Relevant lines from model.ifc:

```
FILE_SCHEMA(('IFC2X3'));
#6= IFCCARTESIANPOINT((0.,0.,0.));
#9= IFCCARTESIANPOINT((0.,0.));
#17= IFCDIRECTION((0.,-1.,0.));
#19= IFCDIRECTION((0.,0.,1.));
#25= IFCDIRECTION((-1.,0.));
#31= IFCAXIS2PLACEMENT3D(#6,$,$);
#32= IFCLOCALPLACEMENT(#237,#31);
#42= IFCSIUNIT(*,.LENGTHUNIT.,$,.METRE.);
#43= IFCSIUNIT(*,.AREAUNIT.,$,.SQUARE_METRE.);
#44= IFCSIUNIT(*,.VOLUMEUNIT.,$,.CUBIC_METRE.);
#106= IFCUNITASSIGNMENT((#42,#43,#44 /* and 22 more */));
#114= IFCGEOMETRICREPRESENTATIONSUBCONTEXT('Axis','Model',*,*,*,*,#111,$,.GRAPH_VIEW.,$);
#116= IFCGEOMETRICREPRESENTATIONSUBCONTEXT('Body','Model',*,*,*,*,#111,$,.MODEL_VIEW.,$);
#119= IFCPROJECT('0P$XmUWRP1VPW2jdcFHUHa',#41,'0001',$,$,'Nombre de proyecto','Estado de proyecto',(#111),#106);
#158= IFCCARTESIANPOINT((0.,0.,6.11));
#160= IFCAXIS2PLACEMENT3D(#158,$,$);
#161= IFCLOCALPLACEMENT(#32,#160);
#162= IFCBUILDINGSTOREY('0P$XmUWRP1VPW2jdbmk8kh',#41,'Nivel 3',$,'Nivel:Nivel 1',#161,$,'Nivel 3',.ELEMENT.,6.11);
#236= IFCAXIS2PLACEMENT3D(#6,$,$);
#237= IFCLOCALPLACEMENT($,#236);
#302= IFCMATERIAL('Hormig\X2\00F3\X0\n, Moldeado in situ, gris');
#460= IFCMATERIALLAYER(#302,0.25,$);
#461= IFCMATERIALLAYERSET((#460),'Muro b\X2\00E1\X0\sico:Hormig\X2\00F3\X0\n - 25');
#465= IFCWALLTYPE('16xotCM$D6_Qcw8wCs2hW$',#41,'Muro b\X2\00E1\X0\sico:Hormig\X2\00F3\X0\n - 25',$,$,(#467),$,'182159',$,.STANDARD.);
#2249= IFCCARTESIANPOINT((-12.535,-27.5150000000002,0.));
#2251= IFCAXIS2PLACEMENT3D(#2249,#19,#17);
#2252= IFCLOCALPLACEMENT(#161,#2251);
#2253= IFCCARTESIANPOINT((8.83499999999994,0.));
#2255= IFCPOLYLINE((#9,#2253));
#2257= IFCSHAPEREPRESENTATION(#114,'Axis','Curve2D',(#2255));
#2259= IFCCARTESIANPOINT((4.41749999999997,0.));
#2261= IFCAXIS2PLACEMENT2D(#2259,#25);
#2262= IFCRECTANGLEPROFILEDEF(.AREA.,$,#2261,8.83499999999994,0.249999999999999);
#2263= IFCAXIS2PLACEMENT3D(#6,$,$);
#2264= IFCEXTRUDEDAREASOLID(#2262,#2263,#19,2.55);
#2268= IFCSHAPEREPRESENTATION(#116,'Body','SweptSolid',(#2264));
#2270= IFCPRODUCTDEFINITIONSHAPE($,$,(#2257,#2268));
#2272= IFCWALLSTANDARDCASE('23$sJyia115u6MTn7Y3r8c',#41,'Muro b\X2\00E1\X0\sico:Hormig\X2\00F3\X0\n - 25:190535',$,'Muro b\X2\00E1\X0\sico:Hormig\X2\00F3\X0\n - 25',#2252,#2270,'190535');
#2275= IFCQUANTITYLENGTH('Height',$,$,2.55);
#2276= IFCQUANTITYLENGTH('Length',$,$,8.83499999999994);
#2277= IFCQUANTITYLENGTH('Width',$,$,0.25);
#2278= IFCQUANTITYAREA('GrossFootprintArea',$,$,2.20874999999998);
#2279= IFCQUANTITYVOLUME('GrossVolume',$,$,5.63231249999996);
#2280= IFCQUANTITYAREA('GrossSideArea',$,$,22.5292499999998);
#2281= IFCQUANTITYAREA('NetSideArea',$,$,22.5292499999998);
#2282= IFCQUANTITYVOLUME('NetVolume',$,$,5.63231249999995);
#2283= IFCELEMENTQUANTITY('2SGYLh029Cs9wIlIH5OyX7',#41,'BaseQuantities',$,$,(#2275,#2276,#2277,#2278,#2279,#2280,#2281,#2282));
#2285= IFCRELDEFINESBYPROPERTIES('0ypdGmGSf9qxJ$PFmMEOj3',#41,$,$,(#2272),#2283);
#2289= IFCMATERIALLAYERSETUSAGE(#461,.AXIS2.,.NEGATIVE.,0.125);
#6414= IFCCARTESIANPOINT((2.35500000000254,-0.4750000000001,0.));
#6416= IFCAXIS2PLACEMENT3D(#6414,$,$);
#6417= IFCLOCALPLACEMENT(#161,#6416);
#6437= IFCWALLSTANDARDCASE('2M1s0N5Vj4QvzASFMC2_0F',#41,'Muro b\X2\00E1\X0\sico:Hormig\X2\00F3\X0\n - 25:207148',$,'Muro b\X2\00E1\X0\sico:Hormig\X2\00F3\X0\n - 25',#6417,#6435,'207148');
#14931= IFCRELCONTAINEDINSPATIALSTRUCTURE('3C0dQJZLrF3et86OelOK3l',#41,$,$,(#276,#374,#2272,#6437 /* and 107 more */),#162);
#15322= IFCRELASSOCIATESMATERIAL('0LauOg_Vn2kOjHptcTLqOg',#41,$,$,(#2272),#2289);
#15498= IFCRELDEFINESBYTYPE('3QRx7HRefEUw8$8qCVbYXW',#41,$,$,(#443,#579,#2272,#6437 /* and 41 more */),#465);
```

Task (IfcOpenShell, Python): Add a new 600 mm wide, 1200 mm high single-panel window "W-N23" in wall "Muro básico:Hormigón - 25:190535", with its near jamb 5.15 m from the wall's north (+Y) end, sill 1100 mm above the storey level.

```python
import numpy as np
import ifcopenshell
import ifcopenshell.api.feature
import ifcopenshell.api.geometry
import ifcopenshell.api.pset
import ifcopenshell.api.root
import ifcopenshell.api.spatial
import ifcopenshell.api.type
import ifcopenshell.geom
import ifcopenshell.util.element
import ifcopenshell.util.placement
import ifcopenshell.util.representation
import ifcopenshell.util.shape
import ifcopenshell.util.unit

model = ifcopenshell.open("model.ifc")
unit_scale = ifcopenshell.util.unit.calculate_unit_scale(model)
area_scale = ifcopenshell.util.unit.calculate_unit_scale(model, "AREAUNIT")
volume_scale = ifcopenshell.util.unit.calculate_unit_scale(model, "VOLUMEUNIT")
settings = ifcopenshell.geom.settings()


def volume(element):
    """Net volume in cubic metres, openings subtracted."""
    shape = ifcopenshell.geom.create_shape(settings, element)
    return ifcopenshell.util.shape.get_volume(shape.geometry)


wall = model.by_guid("23$sJyia115u6MTn7Y3r8c")
storey = ifcopenshell.util.element.get_container(wall, ifc_class="IfcBuildingStorey")
context = ifcopenshell.util.representation.get_context(model, "Model", "Body", "MODEL_VIEW")
before = volume(wall)

width, height, from_end, sill = 0.6, 1.2, 5.15, 1.1  # metres

# The wall runs along its own X axis, and the end named is its -X end.
wall_shape = ifcopenshell.geom.create_shape(settings, wall)
x, y, z = ifcopenshell.util.shape.get_vertices(wall_shape.geometry).T
start = x.min() + from_end
face, thickness = float(y.min()), float(y.max() - y.min())
wall_matrix = ifcopenshell.util.placement.get_local_placement(wall.ObjectPlacement)
level = ifcopenshell.util.placement.get_local_placement(storey.ObjectPlacement)[2, 3]


def in_wall(x, y):
    """Placement at x, y metres in the wall's axes, at sill height."""
    matrix = wall_matrix.copy()
    matrix[:, 3] = wall_matrix @ np.array([x / unit_scale, y / unit_scale, 0.0, 1.0])
    matrix[2, 3] = level + sill / unit_scale
    return matrix


# Opening: a box that overshoots both wall faces by 50 mm.
opening = ifcopenshell.api.root.create_entity(model, ifc_class="IfcOpeningElement")
box = ifcopenshell.api.geometry.add_wall_representation(
    model, context=context, length=width, height=height, thickness=thickness + 0.1
)
ifcopenshell.api.geometry.assign_representation(model, product=opening, representation=box)
ifcopenshell.api.geometry.edit_object_placement(model, product=opening, matrix=in_wall(start, face - 0.05), is_si=False)
ifcopenshell.api.feature.add_feature(model, feature=opening, element=wall)

window = ifcopenshell.api.root.create_entity(model, ifc_class="IfcWindow", name="W-N23")
window.OverallWidth, window.OverallHeight = width / unit_scale, height / unit_scale
body = ifcopenshell.api.geometry.add_window_representation(
    model,
    context=context,
    overall_width=window.OverallWidth,
    overall_height=window.OverallHeight,
    partition_type="SINGLE_PANEL",
)
ifcopenshell.api.geometry.assign_representation(model, product=window, representation=body)
ifcopenshell.api.spatial.assign_container(model, products=[window], relating_structure=storey)
fills = ifcopenshell.api.feature.add_filling(model, opening=opening, element=window)
fills.OwnerHistory = window.OwnerHistory  # required in IFC2X3

# IFC2X3 keeps the operation on the window style.
style = ifcopenshell.api.root.create_entity(model, ifc_class="IfcWindowStyle", name="W-N23")
style.OperationType, style.ConstructionType = "SINGLE_PANEL", "NOTDEFINED"
style.ParameterTakesPrecedence = style.Sizeable = False
ifcopenshell.api.type.assign_type(model, related_objects=[window], relating_type=style)

# Centre the window in the wall's thickness.
ifcopenshell.api.geometry.edit_object_placement(model, product=window, matrix=in_wall(start, face), is_si=False)
window_shape = ifcopenshell.geom.create_shape(settings, window)
depth = ifcopenshell.util.shape.get_vertices(window_shape.geometry)[:, 1]
offset = face + thickness / 2 - (depth.min() + depth.max()) / 2
ifcopenshell.api.geometry.edit_object_placement(model, product=window, matrix=in_wall(start, offset), is_si=False)

after = volume(wall)

# Update the wall's stored quantities.
qto = model.by_id(ifcopenshell.util.element.get_pset(wall, "BaseQuantities", should_inherit=False)["id"])
ifcopenshell.api.pset.edit_qto(model, qto=qto, properties={
    "NetSideArea": after / thickness / area_scale,
    "NetVolume": after / volume_scale,
})

print(f"wall volume {before:.3f} -> {after:.3f} m3")

model.write("model-out.ifc")
```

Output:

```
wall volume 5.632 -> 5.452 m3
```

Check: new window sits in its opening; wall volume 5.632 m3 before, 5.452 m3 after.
